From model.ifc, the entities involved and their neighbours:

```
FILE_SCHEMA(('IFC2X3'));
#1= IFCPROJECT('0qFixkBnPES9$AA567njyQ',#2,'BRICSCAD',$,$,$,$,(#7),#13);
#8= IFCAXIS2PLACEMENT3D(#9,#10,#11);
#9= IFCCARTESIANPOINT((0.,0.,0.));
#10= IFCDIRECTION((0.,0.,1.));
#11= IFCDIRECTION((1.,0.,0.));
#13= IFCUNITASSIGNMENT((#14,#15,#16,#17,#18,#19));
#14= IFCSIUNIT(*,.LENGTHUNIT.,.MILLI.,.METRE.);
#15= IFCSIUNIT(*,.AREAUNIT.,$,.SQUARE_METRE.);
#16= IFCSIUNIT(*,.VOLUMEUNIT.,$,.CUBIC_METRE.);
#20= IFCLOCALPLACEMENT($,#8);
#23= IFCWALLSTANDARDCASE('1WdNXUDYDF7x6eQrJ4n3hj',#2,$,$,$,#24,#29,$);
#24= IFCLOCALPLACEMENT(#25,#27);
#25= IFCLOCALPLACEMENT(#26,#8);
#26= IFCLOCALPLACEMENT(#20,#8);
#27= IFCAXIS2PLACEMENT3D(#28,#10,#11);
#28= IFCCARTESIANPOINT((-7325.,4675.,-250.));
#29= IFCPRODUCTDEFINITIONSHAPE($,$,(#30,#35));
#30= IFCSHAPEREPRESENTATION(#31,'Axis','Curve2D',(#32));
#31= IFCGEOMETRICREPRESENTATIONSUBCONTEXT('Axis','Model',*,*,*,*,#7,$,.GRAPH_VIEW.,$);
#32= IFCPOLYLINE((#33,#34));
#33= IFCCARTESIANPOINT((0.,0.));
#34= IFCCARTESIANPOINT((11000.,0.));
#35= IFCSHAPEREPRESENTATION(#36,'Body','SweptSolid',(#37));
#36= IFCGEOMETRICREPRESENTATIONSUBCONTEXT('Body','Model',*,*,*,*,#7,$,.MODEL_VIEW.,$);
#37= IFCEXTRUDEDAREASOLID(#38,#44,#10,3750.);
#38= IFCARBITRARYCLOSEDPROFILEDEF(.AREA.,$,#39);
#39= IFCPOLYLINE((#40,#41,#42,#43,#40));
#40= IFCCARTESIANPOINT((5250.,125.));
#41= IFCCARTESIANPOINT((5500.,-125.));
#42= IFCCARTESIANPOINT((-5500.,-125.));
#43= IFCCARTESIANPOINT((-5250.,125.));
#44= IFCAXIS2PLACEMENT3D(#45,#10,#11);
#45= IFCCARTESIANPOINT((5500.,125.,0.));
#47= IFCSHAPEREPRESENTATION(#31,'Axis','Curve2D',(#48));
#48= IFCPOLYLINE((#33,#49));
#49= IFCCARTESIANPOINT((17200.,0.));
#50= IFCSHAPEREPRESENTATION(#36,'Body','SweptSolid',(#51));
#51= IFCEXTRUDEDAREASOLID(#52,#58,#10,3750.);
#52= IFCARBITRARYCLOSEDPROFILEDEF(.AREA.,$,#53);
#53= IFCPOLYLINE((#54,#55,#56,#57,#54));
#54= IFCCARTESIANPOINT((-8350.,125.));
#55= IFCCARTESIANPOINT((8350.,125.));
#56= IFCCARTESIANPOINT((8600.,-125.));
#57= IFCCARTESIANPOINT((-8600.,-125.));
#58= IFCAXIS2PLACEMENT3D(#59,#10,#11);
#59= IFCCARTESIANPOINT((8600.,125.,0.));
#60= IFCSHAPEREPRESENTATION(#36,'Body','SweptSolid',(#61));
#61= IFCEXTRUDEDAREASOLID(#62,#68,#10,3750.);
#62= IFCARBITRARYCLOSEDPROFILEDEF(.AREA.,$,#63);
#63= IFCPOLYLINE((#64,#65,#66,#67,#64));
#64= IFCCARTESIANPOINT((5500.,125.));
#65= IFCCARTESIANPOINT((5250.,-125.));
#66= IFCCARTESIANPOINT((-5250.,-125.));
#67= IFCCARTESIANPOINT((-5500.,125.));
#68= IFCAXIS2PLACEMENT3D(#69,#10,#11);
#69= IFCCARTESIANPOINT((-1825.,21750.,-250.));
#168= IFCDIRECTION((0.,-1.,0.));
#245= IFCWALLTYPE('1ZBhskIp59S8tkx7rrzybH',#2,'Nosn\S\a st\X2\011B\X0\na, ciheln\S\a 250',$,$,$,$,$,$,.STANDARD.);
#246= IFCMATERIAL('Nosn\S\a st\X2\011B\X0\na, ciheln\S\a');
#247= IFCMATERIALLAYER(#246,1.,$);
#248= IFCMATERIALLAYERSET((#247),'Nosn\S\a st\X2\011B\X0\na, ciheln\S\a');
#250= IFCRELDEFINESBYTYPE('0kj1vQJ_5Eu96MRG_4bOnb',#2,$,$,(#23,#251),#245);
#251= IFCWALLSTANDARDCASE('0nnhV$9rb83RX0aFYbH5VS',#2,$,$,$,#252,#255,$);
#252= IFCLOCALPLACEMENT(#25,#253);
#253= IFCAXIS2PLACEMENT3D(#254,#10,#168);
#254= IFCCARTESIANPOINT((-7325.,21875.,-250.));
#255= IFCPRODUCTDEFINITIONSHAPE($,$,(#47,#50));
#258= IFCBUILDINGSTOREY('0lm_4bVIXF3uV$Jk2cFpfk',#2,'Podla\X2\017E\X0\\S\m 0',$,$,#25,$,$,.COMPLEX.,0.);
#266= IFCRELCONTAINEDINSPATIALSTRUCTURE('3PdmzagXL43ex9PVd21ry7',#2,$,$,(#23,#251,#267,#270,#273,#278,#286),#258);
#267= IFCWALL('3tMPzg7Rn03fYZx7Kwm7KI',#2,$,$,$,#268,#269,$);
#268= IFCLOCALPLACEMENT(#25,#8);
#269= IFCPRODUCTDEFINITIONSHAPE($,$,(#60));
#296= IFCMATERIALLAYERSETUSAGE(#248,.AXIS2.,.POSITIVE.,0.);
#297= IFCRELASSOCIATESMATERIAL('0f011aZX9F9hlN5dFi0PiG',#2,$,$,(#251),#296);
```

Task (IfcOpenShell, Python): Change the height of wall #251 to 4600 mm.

```python
import ifcopenshell
import ifcopenshell.geom
import ifcopenshell.util.representation
import ifcopenshell.util.shape

model = ifcopenshell.open("model.ifc")
settings = ifcopenshell.geom.settings()


def volume(element):
    """Net volume in cubic metres, openings subtracted."""
    shape = ifcopenshell.geom.create_shape(settings, element)
    return ifcopenshell.util.shape.get_volume(shape.geometry)


wall = model.by_guid("0nnhV$9rb83RX0aFYbH5VS")
before = volume(wall)

body = ifcopenshell.util.representation.get_representation(wall, "Model", "Body")
solid = body.Items[0]
old_height = solid.Depth
solid.Depth = 4600.0
after = volume(wall)

print(f"height {old_height:g} -> {solid.Depth:g}, volume {before:.3f} -> {after:.3f} m3")

model.write("model_v2.ifc")
```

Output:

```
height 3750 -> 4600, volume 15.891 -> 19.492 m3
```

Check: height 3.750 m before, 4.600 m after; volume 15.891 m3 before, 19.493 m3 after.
